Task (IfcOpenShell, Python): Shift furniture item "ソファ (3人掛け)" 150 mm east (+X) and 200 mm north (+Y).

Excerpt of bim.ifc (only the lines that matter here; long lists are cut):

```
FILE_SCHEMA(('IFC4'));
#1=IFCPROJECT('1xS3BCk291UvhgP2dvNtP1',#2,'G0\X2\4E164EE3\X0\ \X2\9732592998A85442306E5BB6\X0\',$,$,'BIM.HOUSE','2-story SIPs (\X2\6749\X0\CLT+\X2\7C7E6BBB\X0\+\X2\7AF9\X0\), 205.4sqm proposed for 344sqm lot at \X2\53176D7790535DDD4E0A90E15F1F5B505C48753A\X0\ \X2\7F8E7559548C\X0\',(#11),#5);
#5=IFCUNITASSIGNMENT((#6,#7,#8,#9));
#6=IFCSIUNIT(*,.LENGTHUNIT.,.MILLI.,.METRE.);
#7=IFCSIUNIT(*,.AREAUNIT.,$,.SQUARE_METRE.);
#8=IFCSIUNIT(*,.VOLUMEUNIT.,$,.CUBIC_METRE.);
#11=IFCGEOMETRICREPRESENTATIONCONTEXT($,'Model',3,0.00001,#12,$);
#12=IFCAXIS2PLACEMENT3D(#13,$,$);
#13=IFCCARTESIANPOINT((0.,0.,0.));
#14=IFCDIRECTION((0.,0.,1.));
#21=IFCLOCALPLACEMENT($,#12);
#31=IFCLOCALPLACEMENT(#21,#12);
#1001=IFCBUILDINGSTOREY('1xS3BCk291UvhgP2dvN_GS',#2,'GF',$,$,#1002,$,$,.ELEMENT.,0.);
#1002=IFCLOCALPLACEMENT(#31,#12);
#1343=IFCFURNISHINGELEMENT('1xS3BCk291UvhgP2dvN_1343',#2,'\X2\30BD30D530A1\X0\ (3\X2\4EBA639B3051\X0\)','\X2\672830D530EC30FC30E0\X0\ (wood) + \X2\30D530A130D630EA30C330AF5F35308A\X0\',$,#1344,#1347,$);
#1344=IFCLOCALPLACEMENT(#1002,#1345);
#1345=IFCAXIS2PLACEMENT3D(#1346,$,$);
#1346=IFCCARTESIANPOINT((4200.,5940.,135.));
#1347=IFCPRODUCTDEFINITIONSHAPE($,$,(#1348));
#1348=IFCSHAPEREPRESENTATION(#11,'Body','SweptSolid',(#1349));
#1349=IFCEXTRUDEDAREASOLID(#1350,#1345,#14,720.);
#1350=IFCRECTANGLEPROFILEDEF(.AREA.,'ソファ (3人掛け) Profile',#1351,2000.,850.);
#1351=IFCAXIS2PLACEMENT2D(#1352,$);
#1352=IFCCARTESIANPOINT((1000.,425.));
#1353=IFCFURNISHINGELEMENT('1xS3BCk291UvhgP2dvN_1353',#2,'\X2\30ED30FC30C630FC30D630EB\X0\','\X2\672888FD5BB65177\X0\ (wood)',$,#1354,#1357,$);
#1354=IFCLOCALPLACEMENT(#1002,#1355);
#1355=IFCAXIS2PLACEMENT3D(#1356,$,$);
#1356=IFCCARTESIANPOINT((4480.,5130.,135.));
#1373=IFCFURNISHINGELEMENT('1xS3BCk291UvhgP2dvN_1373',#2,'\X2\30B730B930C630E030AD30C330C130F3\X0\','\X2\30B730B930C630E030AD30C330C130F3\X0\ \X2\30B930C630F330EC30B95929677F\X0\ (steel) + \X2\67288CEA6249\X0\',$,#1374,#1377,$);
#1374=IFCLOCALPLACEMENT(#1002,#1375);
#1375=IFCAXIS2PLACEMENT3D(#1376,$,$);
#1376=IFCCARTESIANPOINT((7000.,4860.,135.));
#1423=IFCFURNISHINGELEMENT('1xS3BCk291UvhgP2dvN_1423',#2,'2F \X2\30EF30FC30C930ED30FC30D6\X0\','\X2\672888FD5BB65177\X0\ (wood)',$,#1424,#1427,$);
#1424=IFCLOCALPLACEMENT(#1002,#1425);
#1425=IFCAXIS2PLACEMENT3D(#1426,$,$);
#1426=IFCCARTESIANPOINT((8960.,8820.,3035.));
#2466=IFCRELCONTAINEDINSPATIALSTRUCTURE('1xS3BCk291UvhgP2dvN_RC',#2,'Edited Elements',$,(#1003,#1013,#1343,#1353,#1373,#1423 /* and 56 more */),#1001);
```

```python
import ifcopenshell
import ifcopenshell.api.geometry
import ifcopenshell.util.placement
import ifcopenshell.util.unit

model = ifcopenshell.open("bim.ifc")
unit_scale = ifcopenshell.util.unit.calculate_unit_scale(model)

item = model.by_guid("1xS3BCk291UvhgP2dvN_1343")
matrix = ifcopenshell.util.placement.get_local_placement(item.ObjectPlacement)
matrix[0, 3] += 0.15 / unit_scale
matrix[1, 3] += 0.2 / unit_scale
ifcopenshell.api.geometry.edit_object_placement(model, product=item, matrix=matrix, is_si=False)

print(ifcopenshell.util.placement.get_local_placement(item.ObjectPlacement).round(3) + 0.0)

model.write("bim_updated.ifc")
```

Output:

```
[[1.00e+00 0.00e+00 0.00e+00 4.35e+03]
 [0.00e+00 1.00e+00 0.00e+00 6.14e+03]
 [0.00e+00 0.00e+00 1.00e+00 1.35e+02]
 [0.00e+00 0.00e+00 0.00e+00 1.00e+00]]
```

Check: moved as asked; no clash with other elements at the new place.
